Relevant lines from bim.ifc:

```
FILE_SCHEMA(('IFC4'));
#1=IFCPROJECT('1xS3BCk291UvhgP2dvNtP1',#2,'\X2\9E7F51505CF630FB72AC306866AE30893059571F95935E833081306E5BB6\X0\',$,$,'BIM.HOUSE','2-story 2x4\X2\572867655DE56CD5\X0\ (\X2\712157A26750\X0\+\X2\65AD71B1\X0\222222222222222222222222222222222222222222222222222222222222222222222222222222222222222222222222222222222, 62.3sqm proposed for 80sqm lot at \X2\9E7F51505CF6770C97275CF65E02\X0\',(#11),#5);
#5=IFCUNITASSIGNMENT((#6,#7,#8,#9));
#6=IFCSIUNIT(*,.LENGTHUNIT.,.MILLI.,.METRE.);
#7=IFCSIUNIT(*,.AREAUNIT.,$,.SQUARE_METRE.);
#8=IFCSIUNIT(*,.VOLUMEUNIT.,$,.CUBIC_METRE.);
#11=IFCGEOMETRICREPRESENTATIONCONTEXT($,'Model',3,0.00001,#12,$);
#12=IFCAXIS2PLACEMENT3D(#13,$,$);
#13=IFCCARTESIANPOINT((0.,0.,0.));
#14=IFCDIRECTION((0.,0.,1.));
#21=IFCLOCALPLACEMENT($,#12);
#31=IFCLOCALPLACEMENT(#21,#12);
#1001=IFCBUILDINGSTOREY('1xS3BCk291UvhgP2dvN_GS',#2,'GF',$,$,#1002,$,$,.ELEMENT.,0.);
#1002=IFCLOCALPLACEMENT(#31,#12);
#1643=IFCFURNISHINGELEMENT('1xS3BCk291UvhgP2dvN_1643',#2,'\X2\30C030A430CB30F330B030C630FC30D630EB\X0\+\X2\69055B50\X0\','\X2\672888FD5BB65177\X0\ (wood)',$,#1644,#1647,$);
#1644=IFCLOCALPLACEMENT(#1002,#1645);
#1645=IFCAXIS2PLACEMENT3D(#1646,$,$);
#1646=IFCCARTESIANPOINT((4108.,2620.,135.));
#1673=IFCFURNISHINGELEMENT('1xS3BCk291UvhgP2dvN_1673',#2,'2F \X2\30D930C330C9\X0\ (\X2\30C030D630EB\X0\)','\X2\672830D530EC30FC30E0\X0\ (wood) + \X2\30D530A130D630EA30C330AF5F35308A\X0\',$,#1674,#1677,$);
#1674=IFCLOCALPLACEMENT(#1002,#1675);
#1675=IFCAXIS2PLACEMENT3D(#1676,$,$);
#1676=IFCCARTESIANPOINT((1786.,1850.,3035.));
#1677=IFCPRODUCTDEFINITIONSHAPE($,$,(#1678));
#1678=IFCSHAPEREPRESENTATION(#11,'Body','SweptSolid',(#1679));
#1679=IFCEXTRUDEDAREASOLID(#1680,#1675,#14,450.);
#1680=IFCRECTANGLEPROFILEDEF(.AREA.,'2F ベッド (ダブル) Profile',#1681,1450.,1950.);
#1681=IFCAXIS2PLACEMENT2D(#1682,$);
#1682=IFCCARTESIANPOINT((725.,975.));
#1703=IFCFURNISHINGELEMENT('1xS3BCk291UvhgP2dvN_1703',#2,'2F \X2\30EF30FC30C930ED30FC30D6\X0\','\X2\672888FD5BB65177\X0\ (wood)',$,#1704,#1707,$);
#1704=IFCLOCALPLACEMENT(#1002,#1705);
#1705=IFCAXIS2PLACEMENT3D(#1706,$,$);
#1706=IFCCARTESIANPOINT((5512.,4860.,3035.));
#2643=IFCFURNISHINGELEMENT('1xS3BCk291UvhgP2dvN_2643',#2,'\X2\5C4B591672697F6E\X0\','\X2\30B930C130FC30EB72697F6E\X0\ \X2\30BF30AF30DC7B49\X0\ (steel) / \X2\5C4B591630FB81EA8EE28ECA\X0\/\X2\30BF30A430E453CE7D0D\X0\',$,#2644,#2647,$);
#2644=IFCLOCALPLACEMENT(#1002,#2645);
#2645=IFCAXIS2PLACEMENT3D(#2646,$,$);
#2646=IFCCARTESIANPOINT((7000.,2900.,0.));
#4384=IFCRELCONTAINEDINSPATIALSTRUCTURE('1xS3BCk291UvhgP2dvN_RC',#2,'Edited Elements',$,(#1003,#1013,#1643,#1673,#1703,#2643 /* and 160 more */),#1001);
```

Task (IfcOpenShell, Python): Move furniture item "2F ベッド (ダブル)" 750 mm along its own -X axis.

```python
import ifcopenshell
import ifcopenshell.api.geometry
import ifcopenshell.util.placement
import ifcopenshell.util.unit

model = ifcopenshell.open("bim.ifc")
unit_scale = ifcopenshell.util.unit.calculate_unit_scale(model)

item = model.by_guid("1xS3BCk291UvhgP2dvN_1673")
matrix = ifcopenshell.util.placement.get_local_placement(item.ObjectPlacement)
matrix[:3, 3] -= matrix[:3, 0] * 0.75 / unit_scale
ifcopenshell.api.geometry.edit_object_placement(model, product=item, matrix=matrix, is_si=False)

print(ifcopenshell.util.placement.get_local_placement(item.ObjectPlacement).round(3) + 0.0)

model.write("bim_v2.ifc")
```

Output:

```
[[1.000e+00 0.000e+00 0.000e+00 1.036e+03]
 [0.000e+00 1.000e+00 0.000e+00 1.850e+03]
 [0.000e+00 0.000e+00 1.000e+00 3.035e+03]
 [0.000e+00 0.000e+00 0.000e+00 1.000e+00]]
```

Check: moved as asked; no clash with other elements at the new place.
